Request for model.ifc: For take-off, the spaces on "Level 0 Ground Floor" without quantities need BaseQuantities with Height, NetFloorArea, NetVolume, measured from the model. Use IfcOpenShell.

First a look at what the model holds.

```python
import ifcopenshell
import ifcopenshell.util.element
import ifcopenshell.util.unit

model = ifcopenshell.open("model.ifc")
print(model.schema)
for unit_type in ("LENGTHUNIT", "AREAUNIT", "VOLUMEUNIT"):
    print(unit_type, ifcopenshell.util.unit.calculate_unit_scale(model, unit_type))
storey = next(s for s in model.by_type("IfcBuildingStorey") if s.Name == "Level 0 Ground Floor")
spaces = [e for e in ifcopenshell.util.element.get_decomposition(storey) if e.is_a("IfcSpace")]
for e in sorted(spaces, key=lambda e: e.id()):
    print(e.id(), e.is_a(), e.Name, list(ifcopenshell.util.element.get_psets(e, qtos_only=True)), sep=" | ")
```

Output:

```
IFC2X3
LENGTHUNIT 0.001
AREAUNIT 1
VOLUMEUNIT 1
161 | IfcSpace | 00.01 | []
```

```python
import ifcopenshell
import ifcopenshell.api.pset
import ifcopenshell.geom
import ifcopenshell.util.element
import ifcopenshell.util.shape
import ifcopenshell.util.unit

model = ifcopenshell.open("model.ifc")
unit_scale = ifcopenshell.util.unit.calculate_unit_scale(model)
area_scale = ifcopenshell.util.unit.calculate_unit_scale(model, "AREAUNIT")
volume_scale = ifcopenshell.util.unit.calculate_unit_scale(model, "VOLUMEUNIT")
settings = ifcopenshell.geom.settings()

storey = next(s for s in model.by_type("IfcBuildingStorey") if s.Name == "Level 0 Ground Floor")
spaces = [e for e in ifcopenshell.util.element.get_decomposition(storey) if e.is_a("IfcSpace")]

for e in sorted(spaces, key=lambda e: e.id()):
    if ifcopenshell.util.element.get_psets(e, qtos_only=True, should_inherit=False):
        continue
    # Geometry comes back in metres, in the element's own axes.
    shape = ifcopenshell.geom.create_shape(settings, e)
    values = {
        "Height": ifcopenshell.util.shape.get_z(shape.geometry) / unit_scale,
        "NetFloorArea": ifcopenshell.util.shape.get_footprint_area(shape.geometry) / area_scale,
        "NetVolume": ifcopenshell.util.shape.get_volume(shape.geometry) / volume_scale,
    }
    qto = ifcopenshell.api.pset.add_qto(model, product=e, name="BaseQuantities")
    ifcopenshell.api.pset.edit_qto(model, qto=qto, properties=values)
    print(e.id(), {k: round(v, 3) for k, v in values.items()})

model.write("model_rev.ifc")
```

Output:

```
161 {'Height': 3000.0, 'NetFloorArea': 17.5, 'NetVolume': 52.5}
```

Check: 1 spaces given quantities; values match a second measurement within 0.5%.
